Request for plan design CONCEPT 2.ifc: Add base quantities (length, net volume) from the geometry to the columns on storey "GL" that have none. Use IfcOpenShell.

First a look at what the model holds.

```python
import ifcopenshell
import ifcopenshell.util.element
import ifcopenshell.util.unit

model = ifcopenshell.open("plan design CONCEPT 2.ifc")
print(model.schema)
for unit_type in ("LENGTHUNIT", "AREAUNIT", "VOLUMEUNIT"):
    print(unit_type, ifcopenshell.util.unit.calculate_unit_scale(model, unit_type))
storey = next(s for s in model.by_type("IfcBuildingStorey") if s.Name == "GL")
columns = [e for e in ifcopenshell.util.element.get_decomposition(storey) if e.is_a("IfcColumn")]
for e in sorted(columns, key=lambda e: e.id()):
    print(e.id(), e.is_a(), e.Name, list(ifcopenshell.util.element.get_psets(e, qtos_only=True)), sep=" | ")
```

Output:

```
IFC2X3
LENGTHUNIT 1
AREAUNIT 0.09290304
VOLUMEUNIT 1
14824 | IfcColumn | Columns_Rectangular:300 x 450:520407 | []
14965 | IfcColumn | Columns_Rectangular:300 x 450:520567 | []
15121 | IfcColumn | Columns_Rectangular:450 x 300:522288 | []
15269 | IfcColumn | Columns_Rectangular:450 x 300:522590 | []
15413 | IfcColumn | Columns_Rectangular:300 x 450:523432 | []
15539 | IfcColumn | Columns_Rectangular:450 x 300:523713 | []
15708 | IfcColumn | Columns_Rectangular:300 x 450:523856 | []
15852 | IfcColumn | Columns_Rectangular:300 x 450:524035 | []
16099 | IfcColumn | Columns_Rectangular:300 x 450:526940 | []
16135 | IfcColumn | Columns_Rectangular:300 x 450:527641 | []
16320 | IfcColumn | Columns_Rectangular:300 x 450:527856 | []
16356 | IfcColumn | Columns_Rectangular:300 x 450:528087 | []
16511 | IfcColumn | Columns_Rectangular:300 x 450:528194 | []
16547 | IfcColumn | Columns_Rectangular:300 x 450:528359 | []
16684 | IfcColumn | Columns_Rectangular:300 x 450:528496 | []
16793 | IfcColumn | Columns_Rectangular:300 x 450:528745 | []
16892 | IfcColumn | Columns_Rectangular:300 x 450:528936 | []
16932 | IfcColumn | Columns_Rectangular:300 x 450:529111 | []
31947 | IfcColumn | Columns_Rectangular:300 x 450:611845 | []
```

```python
import ifcopenshell
import ifcopenshell.api.pset
import ifcopenshell.geom
import ifcopenshell.util.element
import ifcopenshell.util.shape
import ifcopenshell.util.unit

model = ifcopenshell.open("plan design CONCEPT 2.ifc")
unit_scale = ifcopenshell.util.unit.calculate_unit_scale(model)
volume_scale = ifcopenshell.util.unit.calculate_unit_scale(model, "VOLUMEUNIT")
settings = ifcopenshell.geom.settings()

storey = next(s for s in model.by_type("IfcBuildingStorey") if s.Name == "GL")
columns = [e for e in ifcopenshell.util.element.get_decomposition(storey) if e.is_a("IfcColumn")]

for e in sorted(columns, key=lambda e: e.id()):
    if ifcopenshell.util.element.get_psets(e, qtos_only=True, should_inherit=False):
        continue
    # Geometry comes back in metres, in the element's own axes.
    shape = ifcopenshell.geom.create_shape(settings, e)
    values = {
        "Length": ifcopenshell.util.shape.get_z(shape.geometry) / unit_scale,
        "NetVolume": ifcopenshell.util.shape.get_volume(shape.geometry) / volume_scale,
    }
    qto = ifcopenshell.api.pset.add_qto(model, product=e, name="BaseQuantities")
    ifcopenshell.api.pset.edit_qto(model, qto=qto, properties=values)
    print(e.id(), {k: round(v, 3) for k, v in values.items()})

model.write("plan design CONCEPT 2-out.ifc")
```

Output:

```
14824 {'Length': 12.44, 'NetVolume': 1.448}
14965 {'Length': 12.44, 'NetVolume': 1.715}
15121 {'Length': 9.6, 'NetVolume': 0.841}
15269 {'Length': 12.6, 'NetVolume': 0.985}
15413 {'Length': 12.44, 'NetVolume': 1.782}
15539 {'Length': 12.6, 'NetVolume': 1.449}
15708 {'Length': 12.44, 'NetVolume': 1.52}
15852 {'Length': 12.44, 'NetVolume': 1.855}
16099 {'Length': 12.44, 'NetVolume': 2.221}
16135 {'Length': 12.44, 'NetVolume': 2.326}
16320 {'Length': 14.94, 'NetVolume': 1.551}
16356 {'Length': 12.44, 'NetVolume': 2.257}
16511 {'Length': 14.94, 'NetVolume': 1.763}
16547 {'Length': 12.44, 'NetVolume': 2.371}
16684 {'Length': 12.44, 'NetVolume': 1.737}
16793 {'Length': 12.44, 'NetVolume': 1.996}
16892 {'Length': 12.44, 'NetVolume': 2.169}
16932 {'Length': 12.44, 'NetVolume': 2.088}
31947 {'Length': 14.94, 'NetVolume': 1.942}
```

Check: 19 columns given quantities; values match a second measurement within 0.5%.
